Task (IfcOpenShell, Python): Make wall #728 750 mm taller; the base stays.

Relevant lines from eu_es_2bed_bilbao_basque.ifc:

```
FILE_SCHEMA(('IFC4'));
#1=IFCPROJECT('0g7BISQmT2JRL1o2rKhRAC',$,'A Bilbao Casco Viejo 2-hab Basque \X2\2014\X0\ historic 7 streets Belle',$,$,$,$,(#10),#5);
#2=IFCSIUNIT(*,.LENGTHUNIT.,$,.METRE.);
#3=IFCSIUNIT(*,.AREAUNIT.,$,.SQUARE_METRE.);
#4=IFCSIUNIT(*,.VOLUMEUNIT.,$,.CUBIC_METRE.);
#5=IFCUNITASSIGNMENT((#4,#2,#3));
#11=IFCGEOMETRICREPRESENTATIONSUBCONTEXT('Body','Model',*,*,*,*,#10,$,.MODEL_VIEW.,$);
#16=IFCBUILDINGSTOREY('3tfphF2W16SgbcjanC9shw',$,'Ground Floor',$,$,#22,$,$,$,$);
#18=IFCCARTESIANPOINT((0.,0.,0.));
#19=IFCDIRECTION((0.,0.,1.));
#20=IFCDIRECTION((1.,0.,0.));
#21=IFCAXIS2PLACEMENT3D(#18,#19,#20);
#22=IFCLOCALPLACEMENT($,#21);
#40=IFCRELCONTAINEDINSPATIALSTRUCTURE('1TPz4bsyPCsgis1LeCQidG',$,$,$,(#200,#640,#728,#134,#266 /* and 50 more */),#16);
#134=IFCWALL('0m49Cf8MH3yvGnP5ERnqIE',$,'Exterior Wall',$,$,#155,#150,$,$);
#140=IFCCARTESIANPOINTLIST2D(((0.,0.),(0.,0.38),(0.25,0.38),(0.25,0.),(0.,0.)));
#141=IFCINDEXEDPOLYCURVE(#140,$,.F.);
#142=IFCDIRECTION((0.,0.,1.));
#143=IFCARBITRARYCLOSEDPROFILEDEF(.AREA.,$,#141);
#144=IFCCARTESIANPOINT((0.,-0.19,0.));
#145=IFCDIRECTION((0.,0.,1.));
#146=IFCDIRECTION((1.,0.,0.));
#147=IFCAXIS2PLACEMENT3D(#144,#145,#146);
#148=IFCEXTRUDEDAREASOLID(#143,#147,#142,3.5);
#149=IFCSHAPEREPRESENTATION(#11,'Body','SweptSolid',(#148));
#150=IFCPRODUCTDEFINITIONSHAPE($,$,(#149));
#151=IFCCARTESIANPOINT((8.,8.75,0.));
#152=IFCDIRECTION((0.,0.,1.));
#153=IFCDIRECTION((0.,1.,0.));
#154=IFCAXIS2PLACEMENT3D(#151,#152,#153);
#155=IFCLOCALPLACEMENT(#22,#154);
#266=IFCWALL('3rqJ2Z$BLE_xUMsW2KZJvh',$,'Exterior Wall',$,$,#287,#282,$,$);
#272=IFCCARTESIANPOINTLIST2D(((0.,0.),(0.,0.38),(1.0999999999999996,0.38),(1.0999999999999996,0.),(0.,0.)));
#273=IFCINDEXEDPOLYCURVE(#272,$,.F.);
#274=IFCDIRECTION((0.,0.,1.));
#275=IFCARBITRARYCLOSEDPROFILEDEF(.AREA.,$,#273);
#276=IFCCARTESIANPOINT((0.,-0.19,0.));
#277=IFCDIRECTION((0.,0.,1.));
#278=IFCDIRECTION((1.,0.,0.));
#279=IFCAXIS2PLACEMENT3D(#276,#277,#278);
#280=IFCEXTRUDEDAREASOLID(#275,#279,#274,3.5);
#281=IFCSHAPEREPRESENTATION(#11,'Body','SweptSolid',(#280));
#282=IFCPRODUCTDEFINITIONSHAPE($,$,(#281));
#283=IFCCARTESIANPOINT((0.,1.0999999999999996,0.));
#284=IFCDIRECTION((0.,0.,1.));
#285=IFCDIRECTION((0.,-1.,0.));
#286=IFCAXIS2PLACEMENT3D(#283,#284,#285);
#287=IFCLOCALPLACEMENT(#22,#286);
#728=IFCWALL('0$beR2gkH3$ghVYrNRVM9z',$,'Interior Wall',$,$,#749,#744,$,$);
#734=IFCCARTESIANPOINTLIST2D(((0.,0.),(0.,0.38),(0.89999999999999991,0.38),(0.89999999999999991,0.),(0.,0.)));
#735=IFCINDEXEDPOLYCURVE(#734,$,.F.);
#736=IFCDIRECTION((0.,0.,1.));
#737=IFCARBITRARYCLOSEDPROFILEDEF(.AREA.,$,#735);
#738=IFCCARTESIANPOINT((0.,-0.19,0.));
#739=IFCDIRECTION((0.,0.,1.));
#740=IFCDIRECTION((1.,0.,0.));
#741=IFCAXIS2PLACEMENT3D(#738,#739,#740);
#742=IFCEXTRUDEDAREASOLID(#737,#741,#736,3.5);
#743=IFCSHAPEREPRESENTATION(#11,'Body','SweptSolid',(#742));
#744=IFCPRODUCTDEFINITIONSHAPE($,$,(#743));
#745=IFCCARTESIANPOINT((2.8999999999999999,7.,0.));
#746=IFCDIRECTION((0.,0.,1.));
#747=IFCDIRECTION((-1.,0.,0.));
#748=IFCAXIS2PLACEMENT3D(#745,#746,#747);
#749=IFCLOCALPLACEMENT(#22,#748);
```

```python
import ifcopenshell
import ifcopenshell.geom
import ifcopenshell.util.representation
import ifcopenshell.util.shape
import ifcopenshell.util.unit

model = ifcopenshell.open("eu_es_2bed_bilbao_basque.ifc")
unit_scale = ifcopenshell.util.unit.calculate_unit_scale(model)
settings = ifcopenshell.geom.settings()


def volume(element):
    """Net volume in cubic metres, openings subtracted."""
    shape = ifcopenshell.geom.create_shape(settings, element)
    return ifcopenshell.util.shape.get_volume(shape.geometry)


wall = model.by_guid("0$beR2gkH3$ghVYrNRVM9z")
before = volume(wall)

body = ifcopenshell.util.representation.get_representation(wall, "Model", "Body")
solid = body.Items[0]
old_height = solid.Depth
solid.Depth += 0.75 / unit_scale
after = volume(wall)

print(f"height {old_height:g} -> {solid.Depth:g}, volume {before:.3f} -> {after:.3f} m3")

model.write("eu_es_2bed_bilbao_basque_updated.ifc")
```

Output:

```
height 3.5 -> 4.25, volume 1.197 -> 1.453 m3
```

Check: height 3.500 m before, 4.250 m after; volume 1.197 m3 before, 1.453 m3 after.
